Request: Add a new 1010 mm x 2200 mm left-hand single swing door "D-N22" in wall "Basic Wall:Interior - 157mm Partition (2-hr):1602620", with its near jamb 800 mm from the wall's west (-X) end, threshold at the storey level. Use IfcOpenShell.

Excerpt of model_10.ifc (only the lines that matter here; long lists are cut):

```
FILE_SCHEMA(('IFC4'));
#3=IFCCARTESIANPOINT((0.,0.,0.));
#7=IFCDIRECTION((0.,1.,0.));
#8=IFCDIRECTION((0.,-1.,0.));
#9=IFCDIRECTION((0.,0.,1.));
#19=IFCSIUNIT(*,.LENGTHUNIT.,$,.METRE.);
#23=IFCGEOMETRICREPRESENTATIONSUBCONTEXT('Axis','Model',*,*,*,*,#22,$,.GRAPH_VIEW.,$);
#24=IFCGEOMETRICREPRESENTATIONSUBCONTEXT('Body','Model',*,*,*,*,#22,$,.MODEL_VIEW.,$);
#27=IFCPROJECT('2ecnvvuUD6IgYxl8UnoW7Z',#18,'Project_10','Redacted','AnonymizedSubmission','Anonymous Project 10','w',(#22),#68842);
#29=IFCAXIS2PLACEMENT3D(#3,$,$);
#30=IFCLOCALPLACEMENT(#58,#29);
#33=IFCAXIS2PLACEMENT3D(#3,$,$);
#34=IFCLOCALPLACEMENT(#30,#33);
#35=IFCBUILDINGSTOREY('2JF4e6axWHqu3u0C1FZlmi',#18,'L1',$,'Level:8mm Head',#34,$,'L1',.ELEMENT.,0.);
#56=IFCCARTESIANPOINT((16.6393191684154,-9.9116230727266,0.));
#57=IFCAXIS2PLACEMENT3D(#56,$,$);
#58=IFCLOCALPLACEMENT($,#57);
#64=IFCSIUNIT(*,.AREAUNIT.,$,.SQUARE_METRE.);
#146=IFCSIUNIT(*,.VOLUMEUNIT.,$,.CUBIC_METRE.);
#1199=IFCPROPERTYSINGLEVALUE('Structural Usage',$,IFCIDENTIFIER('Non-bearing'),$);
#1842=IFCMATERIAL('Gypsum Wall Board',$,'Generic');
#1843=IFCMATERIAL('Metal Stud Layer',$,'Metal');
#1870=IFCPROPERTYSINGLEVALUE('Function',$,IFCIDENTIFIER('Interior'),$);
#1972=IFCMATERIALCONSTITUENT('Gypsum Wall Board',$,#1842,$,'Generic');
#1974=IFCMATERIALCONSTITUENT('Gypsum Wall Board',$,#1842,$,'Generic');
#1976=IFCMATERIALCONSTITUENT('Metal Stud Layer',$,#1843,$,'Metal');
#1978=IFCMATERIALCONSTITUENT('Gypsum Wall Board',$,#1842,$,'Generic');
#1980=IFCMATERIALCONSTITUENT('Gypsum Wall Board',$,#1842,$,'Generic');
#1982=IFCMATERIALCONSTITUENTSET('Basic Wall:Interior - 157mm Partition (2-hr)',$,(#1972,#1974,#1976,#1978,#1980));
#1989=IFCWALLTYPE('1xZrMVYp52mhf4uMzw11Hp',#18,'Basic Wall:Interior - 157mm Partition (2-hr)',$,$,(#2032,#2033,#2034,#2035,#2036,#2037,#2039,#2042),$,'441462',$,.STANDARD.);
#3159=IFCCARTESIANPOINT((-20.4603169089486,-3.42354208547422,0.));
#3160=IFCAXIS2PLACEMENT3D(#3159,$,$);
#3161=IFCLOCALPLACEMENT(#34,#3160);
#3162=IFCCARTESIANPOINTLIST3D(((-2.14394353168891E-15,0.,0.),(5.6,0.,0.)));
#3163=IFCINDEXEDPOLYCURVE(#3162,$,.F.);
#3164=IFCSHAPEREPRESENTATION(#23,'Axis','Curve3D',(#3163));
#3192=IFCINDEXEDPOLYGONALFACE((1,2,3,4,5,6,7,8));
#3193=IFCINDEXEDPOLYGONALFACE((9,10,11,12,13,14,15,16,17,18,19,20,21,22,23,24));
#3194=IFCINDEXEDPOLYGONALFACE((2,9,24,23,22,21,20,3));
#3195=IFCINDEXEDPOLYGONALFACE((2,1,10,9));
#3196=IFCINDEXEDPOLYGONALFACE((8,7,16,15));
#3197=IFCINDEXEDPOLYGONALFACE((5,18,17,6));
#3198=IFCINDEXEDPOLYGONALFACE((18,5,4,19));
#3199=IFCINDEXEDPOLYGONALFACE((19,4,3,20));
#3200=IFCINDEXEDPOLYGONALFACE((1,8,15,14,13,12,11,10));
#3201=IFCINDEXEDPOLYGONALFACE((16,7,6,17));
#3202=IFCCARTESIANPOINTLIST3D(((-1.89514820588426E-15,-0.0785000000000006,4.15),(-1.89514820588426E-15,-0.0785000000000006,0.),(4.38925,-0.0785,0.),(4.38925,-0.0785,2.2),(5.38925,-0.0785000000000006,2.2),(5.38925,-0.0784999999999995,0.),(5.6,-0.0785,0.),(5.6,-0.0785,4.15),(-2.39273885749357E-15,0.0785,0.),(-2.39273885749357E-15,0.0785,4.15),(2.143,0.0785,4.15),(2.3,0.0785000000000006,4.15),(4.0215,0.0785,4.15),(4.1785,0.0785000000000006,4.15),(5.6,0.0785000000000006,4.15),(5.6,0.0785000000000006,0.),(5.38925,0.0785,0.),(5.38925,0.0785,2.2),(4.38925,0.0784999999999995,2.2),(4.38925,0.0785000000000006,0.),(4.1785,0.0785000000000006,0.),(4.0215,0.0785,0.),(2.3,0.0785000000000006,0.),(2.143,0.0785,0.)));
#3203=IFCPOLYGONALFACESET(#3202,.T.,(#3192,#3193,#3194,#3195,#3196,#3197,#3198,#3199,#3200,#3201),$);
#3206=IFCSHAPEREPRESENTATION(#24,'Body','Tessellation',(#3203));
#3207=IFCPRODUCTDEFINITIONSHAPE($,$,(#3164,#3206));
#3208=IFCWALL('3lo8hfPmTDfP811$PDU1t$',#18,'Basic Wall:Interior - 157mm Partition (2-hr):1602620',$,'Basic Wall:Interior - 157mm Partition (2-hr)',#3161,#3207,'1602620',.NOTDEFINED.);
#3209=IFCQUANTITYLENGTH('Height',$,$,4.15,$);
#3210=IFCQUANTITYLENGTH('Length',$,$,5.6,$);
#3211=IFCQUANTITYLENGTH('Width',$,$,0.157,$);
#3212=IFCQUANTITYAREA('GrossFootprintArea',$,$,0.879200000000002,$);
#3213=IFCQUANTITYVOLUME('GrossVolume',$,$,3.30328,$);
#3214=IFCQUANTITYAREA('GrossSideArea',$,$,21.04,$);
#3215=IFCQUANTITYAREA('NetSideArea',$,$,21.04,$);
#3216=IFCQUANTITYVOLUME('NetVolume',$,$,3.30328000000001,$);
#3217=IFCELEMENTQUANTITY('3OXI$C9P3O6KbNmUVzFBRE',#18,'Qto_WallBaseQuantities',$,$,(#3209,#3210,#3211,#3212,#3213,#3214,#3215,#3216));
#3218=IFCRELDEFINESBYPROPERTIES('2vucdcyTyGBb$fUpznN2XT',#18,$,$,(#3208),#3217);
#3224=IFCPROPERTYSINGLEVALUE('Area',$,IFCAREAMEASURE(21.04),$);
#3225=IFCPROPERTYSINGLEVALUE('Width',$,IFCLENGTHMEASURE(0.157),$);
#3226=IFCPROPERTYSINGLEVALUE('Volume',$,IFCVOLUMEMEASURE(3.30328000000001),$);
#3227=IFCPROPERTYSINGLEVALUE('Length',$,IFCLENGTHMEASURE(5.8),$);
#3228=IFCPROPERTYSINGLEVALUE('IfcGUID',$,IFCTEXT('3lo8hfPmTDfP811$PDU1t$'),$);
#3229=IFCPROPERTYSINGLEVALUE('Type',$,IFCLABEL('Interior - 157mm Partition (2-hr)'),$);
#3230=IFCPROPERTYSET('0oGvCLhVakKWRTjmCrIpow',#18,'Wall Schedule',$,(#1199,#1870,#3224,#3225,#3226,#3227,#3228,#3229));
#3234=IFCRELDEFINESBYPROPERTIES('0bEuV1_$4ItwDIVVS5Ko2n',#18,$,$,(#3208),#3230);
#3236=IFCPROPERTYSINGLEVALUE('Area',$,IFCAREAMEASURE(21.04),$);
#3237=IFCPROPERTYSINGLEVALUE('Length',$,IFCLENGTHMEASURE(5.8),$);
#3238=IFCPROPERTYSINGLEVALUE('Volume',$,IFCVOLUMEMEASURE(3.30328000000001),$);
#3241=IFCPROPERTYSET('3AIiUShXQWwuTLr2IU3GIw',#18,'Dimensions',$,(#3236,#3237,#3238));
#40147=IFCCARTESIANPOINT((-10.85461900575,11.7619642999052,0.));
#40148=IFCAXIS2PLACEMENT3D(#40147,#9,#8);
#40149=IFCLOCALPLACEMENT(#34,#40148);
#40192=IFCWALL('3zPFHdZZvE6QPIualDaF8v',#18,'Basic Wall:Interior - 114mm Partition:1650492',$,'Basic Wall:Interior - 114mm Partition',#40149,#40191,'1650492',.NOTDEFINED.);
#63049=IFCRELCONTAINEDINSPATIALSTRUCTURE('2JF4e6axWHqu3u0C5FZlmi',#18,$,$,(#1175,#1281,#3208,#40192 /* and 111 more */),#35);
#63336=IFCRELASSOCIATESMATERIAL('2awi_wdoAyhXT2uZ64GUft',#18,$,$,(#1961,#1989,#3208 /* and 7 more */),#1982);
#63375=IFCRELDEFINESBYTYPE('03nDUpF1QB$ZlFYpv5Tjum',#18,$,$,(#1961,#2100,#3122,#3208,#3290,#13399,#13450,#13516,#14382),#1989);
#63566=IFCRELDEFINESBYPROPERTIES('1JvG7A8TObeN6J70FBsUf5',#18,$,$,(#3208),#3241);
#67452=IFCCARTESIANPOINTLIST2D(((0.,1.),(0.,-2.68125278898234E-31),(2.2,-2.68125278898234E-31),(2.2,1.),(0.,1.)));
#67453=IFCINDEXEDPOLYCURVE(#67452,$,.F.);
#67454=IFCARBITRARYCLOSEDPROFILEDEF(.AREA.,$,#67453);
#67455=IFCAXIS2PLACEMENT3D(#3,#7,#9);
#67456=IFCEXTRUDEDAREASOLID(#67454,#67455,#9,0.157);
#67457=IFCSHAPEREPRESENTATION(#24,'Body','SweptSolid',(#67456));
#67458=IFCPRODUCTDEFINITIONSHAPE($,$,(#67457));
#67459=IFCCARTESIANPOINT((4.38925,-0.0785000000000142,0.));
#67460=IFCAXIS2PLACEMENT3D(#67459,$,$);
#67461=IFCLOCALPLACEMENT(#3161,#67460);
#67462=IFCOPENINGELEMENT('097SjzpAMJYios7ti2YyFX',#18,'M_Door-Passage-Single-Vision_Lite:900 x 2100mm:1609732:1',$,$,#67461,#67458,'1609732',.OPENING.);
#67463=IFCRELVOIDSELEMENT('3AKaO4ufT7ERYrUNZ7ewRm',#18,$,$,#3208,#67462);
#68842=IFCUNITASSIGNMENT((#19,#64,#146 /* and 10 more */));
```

```python
import numpy as np
import ifcopenshell
import ifcopenshell.api.feature
import ifcopenshell.api.geometry
import ifcopenshell.api.pset
import ifcopenshell.api.root
import ifcopenshell.api.spatial
import ifcopenshell.geom
import ifcopenshell.util.element
import ifcopenshell.util.placement
import ifcopenshell.util.representation
import ifcopenshell.util.shape
import ifcopenshell.util.unit

model = ifcopenshell.open("model_10.ifc")
unit_scale = ifcopenshell.util.unit.calculate_unit_scale(model)
area_scale = ifcopenshell.util.unit.calculate_unit_scale(model, "AREAUNIT")
volume_scale = ifcopenshell.util.unit.calculate_unit_scale(model, "VOLUMEUNIT")
settings = ifcopenshell.geom.settings()


def volume(element):
    """Net volume in cubic metres, openings subtracted."""
    shape = ifcopenshell.geom.create_shape(settings, element)
    return ifcopenshell.util.shape.get_volume(shape.geometry)


wall = model.by_guid("3lo8hfPmTDfP811$PDU1t$")
storey = ifcopenshell.util.element.get_container(wall, ifc_class="IfcBuildingStorey")
context = ifcopenshell.util.representation.get_context(model, "Model", "Body", "MODEL_VIEW")
before = volume(wall)

width, height, from_end, sill = 1.01, 2.2, 0.8, 0.0  # metres

# The wall runs along its own X axis, and the end named is its -X end.
wall_shape = ifcopenshell.geom.create_shape(settings, wall)
x, y, z = ifcopenshell.util.shape.get_vertices(wall_shape.geometry).T
start = x.min() + from_end
face, thickness = float(y.min()), float(y.max() - y.min())
wall_matrix = ifcopenshell.util.placement.get_local_placement(wall.ObjectPlacement)
level = ifcopenshell.util.placement.get_local_placement(storey.ObjectPlacement)[2, 3]


def in_wall(x, y):
    """Placement at x, y metres in the wall's axes, at sill height."""
    matrix = wall_matrix.copy()
    matrix[:, 3] = wall_matrix @ np.array([x / unit_scale, y / unit_scale, 0.0, 1.0])
    matrix[2, 3] = level + sill / unit_scale
    return matrix


# Opening: a box that overshoots both wall faces by 50 mm.
opening = ifcopenshell.api.root.create_entity(model, ifc_class="IfcOpeningElement", predefined_type="OPENING")
box = ifcopenshell.api.geometry.add_wall_representation(
    model, context=context, length=width, height=height, thickness=thickness + 0.1
)
ifcopenshell.api.geometry.assign_representation(model, product=opening, representation=box)
ifcopenshell.api.geometry.edit_object_placement(model, product=opening, matrix=in_wall(start, face - 0.05), is_si=False)
ifcopenshell.api.feature.add_feature(model, feature=opening, element=wall)

door = ifcopenshell.api.root.create_entity(model, ifc_class="IfcDoor", name="D-N22", predefined_type="DOOR")
door.OverallWidth, door.OverallHeight = width / unit_scale, height / unit_scale
door.OperationType = "SINGLE_SWING_LEFT"
body = ifcopenshell.api.geometry.add_door_representation(
    model,
    context=context,
    overall_width=door.OverallWidth,
    overall_height=door.OverallHeight,
    operation_type="SINGLE_SWING_LEFT",
    lining_properties={"LiningDepth": thickness / unit_scale, "ThresholdDepth": thickness / unit_scale},
)
ifcopenshell.api.geometry.assign_representation(model, product=door, representation=body)
ifcopenshell.api.spatial.assign_container(model, products=[door], relating_structure=storey)
ifcopenshell.api.feature.add_filling(model, opening=opening, element=door)

# The lining spans the wall, so the door starts at the wall face.
ifcopenshell.api.geometry.edit_object_placement(model, product=door, matrix=in_wall(start, face), is_si=False)

after = volume(wall)

# Update the wall's stored quantities.
qto = model.by_id(ifcopenshell.util.element.get_pset(wall, "Qto_WallBaseQuantities", should_inherit=False)["id"])
ifcopenshell.api.pset.edit_qto(model, qto=qto, properties={
    "NetSideArea": after / thickness / area_scale,
    "NetVolume": after / volume_scale,
})
pset = model.by_id(ifcopenshell.util.element.get_pset(wall, "Wall Schedule", should_inherit=False)["id"])
ifcopenshell.api.pset.edit_pset(model, pset=pset, properties={
    "Area": model.create_entity("IfcAreaMeasure", after / thickness / area_scale),
    "Volume": model.create_entity("IfcVolumeMeasure", after / volume_scale),
})
pset = model.by_id(ifcopenshell.util.element.get_pset(wall, "Dimensions", should_inherit=False)["id"])
ifcopenshell.api.pset.edit_pset(model, pset=pset, properties={
    "Area": model.create_entity("IfcAreaMeasure", after / thickness / area_scale),
    "Volume": model.create_entity("IfcVolumeMeasure", after / volume_scale),
})

print(f"wall volume {before:.3f} -> {after:.3f} m3")

model.write("model_10_updated.ifc")
```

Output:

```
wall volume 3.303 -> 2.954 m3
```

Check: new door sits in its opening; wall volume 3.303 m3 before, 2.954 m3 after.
